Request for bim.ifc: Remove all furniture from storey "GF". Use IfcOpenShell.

First a look at what the model holds.

```python
import ifcopenshell
import ifcopenshell.util.element

model = ifcopenshell.open("bim.ifc")
print(model.schema)
storey = next(s for s in model.by_type("IfcBuildingStorey") if s.Name == "GF")
furniture = [e for e in ifcopenshell.util.element.get_decomposition(storey) if e.is_a("IfcFurnishingElement")]
seen = {}
for e in furniture:
    element_type = ifcopenshell.util.element.get_type(e)
    name = element_type.Name if element_type not in (None, e) else None
    seen[name] = seen.get(name, 0) + 1
for name, count in sorted(seen.items(), key=str):
    print(count, "x", name)
```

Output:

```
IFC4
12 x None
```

```python
import ifcopenshell
import ifcopenshell.api.root
import ifcopenshell.util.element

model = ifcopenshell.open("bim.ifc")

storey = next(s for s in model.by_type("IfcBuildingStorey") if s.Name == "GF")
furniture = [e for e in ifcopenshell.util.element.get_decomposition(storey) if e.is_a("IfcFurnishingElement")]

for e in furniture:
    ifcopenshell.api.root.remove_product(model, product=e)
print(len(furniture), "removed")

model.write("bim_v2.ifc")
```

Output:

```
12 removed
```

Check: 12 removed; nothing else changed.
